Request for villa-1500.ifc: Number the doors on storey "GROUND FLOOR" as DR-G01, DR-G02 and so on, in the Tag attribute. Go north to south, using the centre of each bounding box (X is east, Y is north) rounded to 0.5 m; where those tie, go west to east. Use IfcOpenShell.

First a look at what the model holds.

```python
import ifcopenshell
import ifcopenshell.util.element
import ifcopenshell.util.placement

model = ifcopenshell.open("villa-1500.ifc")
print(model.schema)
storey = next(s for s in model.by_type("IfcBuildingStorey") if s.Name == "GROUND FLOOR")
doors = [e for e in ifcopenshell.util.element.get_decomposition(storey) if e.is_a("IfcDoor")]
for e in sorted(doors, key=lambda e: e.id()):
    origin = ifcopenshell.util.placement.get_local_placement(e.ObjectPlacement)[:3, 3]
    print(e.id(), e.Tag, e.Name, origin.round(2) + 0.0, sep=" | ")
```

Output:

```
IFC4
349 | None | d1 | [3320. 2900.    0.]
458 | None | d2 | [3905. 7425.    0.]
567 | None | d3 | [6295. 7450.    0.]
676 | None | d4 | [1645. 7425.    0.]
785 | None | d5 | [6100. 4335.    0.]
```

```python
import ifcopenshell
import ifcopenshell.geom
import ifcopenshell.util.element
import ifcopenshell.util.shape

model = ifcopenshell.open("villa-1500.ifc")
settings = ifcopenshell.geom.settings()
settings.set("use-world-coords", True)


def centre(element):
    shape = ifcopenshell.geom.create_shape(settings, element)
    return ifcopenshell.util.shape.get_bbox_centroid(shape.geometry)


storey = next(s for s in model.by_type("IfcBuildingStorey") if s.Name == "GROUND FLOOR")
doors = [e for e in ifcopenshell.util.element.get_decomposition(storey) if e.is_a("IfcDoor")]

# Insertion points can sit at a corner or the storey origin, so sort by the geometry (in metres).
centres = {e: centre(e) for e in doors}
doors.sort(key=lambda e: (-round(centres[e][1] / 0.5), centres[e][0]))

for i, e in enumerate(doors, start=1):
    number = f"DR-G{i:02d}"
    e.Tag = number
    print(e.id(), number)

model.write("villa-1500-out.ifc")
```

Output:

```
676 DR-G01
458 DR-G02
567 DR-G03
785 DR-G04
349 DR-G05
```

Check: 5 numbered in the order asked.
